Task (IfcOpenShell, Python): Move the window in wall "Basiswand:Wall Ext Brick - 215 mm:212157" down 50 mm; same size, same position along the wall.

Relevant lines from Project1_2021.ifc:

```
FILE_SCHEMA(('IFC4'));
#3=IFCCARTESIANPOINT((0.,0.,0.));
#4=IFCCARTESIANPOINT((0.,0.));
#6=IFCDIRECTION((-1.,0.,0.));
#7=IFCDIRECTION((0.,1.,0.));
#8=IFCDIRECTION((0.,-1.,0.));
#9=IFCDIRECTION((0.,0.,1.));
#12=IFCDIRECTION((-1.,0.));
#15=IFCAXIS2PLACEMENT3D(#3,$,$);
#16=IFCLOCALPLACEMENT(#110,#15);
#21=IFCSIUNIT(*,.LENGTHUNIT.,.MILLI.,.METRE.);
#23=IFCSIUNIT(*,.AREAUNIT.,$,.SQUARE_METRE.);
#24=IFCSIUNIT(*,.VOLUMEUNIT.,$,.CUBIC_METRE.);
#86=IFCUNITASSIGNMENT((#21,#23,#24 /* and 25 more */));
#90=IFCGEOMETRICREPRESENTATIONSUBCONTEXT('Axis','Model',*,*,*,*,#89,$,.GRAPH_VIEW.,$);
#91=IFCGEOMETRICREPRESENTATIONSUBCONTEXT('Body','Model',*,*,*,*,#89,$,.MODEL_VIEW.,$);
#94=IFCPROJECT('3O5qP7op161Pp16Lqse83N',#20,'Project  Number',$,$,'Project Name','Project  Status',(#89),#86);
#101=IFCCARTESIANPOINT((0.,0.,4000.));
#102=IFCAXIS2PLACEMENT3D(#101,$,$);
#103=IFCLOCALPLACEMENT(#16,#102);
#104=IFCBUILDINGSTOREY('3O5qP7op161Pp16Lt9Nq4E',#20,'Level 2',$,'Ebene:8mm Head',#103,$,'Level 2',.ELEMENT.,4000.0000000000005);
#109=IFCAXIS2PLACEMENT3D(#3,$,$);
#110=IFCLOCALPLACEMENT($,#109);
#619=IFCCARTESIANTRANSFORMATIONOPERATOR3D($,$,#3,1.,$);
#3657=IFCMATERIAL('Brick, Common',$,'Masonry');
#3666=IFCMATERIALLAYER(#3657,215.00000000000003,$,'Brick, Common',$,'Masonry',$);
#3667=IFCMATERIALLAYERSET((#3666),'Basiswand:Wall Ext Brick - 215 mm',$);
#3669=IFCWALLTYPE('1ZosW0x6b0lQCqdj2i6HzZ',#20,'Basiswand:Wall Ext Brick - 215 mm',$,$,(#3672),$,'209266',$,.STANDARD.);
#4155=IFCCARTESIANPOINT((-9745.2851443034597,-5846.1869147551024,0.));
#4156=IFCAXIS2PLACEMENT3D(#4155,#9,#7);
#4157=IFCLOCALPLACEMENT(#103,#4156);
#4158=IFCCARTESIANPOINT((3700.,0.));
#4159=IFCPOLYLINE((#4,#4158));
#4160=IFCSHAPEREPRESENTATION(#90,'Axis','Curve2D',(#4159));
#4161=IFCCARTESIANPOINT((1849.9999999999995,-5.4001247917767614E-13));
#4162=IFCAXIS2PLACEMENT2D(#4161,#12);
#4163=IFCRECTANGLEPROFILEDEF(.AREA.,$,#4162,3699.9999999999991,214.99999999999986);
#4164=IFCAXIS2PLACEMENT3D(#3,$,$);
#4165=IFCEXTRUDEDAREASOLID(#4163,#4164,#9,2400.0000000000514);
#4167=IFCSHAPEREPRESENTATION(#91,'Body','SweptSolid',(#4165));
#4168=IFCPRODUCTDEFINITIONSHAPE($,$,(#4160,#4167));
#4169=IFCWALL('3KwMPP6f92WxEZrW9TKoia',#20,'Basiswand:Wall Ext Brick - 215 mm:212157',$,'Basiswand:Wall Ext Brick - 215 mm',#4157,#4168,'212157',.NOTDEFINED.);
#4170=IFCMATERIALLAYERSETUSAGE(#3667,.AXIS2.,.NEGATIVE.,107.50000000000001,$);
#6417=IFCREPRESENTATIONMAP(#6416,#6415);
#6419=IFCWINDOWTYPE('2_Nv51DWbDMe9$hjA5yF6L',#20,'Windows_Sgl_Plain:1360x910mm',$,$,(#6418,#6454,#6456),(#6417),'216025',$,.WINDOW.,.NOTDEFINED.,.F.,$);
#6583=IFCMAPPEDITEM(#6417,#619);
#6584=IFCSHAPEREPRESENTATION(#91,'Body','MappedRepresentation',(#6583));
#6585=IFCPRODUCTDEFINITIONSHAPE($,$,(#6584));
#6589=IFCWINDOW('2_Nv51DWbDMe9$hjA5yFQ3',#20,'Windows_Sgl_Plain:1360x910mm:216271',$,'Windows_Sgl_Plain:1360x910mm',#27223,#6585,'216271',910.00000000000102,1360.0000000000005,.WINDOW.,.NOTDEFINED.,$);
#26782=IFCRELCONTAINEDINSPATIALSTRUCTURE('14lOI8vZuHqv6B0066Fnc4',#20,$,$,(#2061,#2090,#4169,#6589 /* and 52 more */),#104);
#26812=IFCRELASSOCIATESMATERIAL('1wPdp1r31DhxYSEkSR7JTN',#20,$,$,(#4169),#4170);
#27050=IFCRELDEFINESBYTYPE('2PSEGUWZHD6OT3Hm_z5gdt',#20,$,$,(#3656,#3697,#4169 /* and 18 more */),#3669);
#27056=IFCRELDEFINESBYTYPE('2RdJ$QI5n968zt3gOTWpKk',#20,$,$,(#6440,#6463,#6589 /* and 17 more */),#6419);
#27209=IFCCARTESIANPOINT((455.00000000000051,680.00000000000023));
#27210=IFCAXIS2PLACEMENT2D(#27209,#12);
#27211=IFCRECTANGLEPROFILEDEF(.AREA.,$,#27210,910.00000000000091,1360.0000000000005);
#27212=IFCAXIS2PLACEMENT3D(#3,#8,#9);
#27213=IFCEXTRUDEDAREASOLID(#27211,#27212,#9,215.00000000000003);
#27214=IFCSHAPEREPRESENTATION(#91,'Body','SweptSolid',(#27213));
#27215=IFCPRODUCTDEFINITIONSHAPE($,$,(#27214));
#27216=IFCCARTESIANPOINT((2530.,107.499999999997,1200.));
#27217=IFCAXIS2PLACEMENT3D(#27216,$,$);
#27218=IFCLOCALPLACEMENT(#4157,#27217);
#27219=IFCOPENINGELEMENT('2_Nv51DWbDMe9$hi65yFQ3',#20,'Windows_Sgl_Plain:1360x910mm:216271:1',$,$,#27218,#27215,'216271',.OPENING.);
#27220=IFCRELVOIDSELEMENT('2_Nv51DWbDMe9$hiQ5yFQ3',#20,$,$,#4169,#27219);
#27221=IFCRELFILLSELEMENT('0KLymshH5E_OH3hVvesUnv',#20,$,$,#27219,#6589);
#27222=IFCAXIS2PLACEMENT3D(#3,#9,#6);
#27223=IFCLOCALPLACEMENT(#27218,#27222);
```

```python
import numpy as np
import ifcopenshell
import ifcopenshell.api.geometry
import ifcopenshell.util.placement
import ifcopenshell.util.unit

model = ifcopenshell.open("Project1_2021.ifc")
unit_scale = ifcopenshell.util.unit.calculate_unit_scale(model)

window = model.by_guid("2_Nv51DWbDMe9$hjA5yFQ3")
opening = window.FillsVoids[0].RelatingOpeningElement
dz = -0.05 / unit_scale

shift = np.array([0.0, 0.0, dz])
# The window is placed relative to its opening, so it follows when the opening moves.
matrix = ifcopenshell.util.placement.get_local_placement(opening.ObjectPlacement)
matrix[:3, 3] += shift
ifcopenshell.api.geometry.edit_object_placement(
    model, product=opening, matrix=matrix, is_si=False, should_transform_children=True
)

print(f"moved by {dz * unit_scale:+.3f} m")

model.write("Project1_2021-out.ifc")
```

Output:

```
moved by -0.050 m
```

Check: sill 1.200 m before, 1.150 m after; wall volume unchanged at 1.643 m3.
